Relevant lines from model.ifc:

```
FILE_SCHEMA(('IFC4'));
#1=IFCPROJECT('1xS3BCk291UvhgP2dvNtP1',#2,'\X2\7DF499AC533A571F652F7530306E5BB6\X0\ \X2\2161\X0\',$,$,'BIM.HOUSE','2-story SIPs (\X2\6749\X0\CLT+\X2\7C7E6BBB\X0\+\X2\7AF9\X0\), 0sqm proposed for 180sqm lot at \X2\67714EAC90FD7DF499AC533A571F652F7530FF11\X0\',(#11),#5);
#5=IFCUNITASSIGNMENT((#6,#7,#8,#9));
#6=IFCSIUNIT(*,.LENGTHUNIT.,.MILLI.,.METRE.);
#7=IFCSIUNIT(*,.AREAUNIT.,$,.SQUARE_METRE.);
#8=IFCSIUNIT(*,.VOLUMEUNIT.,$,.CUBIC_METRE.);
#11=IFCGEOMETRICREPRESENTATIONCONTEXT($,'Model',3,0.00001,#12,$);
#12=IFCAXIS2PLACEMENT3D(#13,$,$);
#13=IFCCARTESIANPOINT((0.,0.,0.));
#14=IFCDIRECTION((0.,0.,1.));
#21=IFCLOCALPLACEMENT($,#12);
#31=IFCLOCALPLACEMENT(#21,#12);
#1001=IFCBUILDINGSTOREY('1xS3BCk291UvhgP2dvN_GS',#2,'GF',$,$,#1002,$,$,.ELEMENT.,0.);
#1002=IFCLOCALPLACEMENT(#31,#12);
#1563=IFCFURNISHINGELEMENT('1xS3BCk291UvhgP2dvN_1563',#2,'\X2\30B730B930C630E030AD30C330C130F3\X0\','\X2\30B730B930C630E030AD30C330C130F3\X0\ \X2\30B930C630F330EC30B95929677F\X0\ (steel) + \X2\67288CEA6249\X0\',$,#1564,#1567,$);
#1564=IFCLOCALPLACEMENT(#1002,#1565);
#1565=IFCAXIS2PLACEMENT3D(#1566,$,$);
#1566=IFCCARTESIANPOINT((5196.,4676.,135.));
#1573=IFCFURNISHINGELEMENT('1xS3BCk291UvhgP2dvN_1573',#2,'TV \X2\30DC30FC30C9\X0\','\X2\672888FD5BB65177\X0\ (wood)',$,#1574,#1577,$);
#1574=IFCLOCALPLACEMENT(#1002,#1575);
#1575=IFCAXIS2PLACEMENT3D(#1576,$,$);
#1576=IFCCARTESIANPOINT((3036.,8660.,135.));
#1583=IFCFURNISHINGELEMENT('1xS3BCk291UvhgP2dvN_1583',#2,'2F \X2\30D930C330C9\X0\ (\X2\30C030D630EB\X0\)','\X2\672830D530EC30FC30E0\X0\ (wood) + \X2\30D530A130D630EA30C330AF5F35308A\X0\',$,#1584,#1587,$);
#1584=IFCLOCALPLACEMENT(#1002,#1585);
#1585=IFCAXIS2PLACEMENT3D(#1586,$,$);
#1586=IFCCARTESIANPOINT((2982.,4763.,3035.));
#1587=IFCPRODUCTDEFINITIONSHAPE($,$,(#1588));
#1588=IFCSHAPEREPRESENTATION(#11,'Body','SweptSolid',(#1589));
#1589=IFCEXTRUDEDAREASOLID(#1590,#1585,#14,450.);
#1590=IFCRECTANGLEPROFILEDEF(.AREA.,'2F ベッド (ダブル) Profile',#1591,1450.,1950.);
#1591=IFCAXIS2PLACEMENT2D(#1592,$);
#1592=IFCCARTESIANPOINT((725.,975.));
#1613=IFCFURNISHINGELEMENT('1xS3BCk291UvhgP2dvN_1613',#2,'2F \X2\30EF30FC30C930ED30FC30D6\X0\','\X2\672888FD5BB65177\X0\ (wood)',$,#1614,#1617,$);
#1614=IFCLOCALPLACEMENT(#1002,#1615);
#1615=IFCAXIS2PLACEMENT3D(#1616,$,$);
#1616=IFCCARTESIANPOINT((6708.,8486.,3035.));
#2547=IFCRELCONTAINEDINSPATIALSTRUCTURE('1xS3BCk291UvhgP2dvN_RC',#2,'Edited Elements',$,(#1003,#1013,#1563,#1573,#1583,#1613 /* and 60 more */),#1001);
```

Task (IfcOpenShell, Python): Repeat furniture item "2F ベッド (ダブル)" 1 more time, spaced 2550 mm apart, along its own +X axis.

```python
import ifcopenshell
import ifcopenshell.api.geometry
import ifcopenshell.api.root
import ifcopenshell.util.element
import ifcopenshell.util.placement
import ifcopenshell.util.unit

model = ifcopenshell.open("model.ifc")
unit_scale = ifcopenshell.util.unit.calculate_unit_scale(model)


def reuse_history(source, copy):
    """copy_class also copies each property set's owner history, people and application; keep the originals."""
    for rel in copy.IsDefinedBy:
        if rel.is_a("IfcRelDefinesByProperties") and (history := rel.RelatingPropertyDefinition.OwnerHistory):
            rel.RelatingPropertyDefinition.OwnerHistory = source.OwnerHistory
            ifcopenshell.util.element.remove_deep2(model, history)


source = model.by_guid("1xS3BCk291UvhgP2dvN_1583")
base = ifcopenshell.util.placement.get_local_placement(source.ObjectPlacement)
step = base[:3, 0] * 2.55 / unit_scale

for i in range(1, 2):
    copy = ifcopenshell.api.root.copy_class(model, product=source)
    copy.Representation = ifcopenshell.util.element.copy_deep(
        model, source.Representation, exclude=["IfcGeometricRepresentationContext", "IfcRepresentationMap"]
    )
    reuse_history(source, copy)
    matrix = base.copy()
    matrix[:3, 3] += i * step
    print("added at", matrix[:3, 3].round(3) + 0.0)
    ifcopenshell.api.geometry.edit_object_placement(model, product=copy, matrix=matrix, is_si=False)

model.write("model_rev.ifc")
```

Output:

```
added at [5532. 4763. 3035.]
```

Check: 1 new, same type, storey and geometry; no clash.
